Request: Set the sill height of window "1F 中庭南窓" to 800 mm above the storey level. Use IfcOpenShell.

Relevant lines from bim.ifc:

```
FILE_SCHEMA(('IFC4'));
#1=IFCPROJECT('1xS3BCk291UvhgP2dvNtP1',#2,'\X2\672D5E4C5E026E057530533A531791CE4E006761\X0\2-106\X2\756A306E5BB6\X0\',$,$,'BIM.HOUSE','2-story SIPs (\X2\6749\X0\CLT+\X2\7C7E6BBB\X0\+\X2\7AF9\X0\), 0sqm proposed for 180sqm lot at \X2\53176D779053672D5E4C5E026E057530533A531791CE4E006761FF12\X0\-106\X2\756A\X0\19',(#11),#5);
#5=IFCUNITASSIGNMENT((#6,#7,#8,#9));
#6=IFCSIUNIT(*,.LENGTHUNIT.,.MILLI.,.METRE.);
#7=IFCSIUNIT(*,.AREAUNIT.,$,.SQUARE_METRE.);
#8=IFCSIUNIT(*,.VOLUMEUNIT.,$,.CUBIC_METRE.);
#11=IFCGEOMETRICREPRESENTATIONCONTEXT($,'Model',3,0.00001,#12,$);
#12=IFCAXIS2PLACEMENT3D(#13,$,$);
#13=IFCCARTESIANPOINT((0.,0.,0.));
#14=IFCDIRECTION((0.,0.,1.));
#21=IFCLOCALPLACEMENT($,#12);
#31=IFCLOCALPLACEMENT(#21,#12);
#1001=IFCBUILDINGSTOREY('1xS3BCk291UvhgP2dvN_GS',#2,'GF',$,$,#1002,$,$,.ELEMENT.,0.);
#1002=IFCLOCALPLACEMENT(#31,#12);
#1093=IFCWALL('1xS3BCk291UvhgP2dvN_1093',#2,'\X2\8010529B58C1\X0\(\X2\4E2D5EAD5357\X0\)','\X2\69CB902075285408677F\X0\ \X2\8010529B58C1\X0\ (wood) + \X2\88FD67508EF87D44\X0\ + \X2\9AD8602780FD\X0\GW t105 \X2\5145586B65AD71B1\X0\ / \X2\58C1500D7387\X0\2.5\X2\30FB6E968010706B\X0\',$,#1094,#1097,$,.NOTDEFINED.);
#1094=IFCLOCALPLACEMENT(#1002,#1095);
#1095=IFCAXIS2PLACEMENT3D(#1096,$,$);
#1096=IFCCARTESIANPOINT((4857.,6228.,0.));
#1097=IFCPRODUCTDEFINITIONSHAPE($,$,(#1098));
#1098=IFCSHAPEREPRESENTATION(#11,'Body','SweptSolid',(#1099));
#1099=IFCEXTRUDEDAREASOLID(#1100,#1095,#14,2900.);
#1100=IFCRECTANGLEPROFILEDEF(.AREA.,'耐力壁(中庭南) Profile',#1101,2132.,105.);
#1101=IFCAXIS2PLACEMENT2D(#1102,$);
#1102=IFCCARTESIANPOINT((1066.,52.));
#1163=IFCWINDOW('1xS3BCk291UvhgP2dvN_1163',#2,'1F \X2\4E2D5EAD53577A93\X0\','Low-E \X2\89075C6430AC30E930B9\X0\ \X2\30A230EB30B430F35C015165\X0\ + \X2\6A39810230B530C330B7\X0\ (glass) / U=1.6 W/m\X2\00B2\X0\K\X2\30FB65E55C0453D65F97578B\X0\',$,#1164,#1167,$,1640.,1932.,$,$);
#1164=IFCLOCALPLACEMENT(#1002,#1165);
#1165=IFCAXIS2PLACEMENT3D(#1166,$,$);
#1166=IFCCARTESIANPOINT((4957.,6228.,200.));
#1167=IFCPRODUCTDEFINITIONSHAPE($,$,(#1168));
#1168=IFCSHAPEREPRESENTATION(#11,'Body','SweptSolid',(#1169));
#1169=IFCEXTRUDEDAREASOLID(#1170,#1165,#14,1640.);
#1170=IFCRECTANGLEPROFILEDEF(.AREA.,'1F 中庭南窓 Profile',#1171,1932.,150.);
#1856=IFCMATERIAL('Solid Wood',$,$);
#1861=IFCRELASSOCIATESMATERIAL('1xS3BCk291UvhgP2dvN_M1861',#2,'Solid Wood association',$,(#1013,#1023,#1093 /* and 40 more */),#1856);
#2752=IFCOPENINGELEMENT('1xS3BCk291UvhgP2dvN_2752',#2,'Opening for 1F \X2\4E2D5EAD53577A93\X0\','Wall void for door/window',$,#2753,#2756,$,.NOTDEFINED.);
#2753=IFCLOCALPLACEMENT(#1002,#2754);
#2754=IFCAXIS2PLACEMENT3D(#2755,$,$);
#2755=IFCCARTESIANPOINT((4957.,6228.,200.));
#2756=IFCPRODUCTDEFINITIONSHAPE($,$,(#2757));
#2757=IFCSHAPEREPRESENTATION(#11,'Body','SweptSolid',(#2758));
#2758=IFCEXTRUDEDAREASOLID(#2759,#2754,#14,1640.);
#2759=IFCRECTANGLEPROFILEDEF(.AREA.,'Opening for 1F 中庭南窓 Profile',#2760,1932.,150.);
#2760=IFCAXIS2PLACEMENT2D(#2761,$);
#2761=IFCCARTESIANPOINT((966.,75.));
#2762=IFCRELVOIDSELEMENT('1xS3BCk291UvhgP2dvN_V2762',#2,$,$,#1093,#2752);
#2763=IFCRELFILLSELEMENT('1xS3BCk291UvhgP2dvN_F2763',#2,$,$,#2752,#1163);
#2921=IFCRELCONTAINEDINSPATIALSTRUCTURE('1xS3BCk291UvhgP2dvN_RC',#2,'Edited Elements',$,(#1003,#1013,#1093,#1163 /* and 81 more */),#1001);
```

```python
import numpy as np
import ifcopenshell
import ifcopenshell.api.geometry
import ifcopenshell.geom
import ifcopenshell.util.element
import ifcopenshell.util.placement
import ifcopenshell.util.shape
import ifcopenshell.util.unit

model = ifcopenshell.open("bim.ifc")
unit_scale = ifcopenshell.util.unit.calculate_unit_scale(model)

window = model.by_guid("1xS3BCk291UvhgP2dvN_1163")
opening = window.FillsVoids[0].RelatingOpeningElement
storey = ifcopenshell.util.element.get_container(window, ifc_class="IfcBuildingStorey")
level = ifcopenshell.util.placement.get_local_placement(storey.ObjectPlacement)[2, 3]

# The opening's origin need not be at the sill, so measure its lowest point.
shape = ifcopenshell.geom.create_shape(ifcopenshell.geom.settings(), opening)
bottom = ifcopenshell.util.shape.get_shape_bottom_elevation(shape, shape.geometry) / unit_scale
dz = level + 0.8 / unit_scale - bottom

shift = np.array([0.0, 0.0, dz])
# The window is not placed relative to its opening, so move both.
for product in (opening, window):
    matrix = ifcopenshell.util.placement.get_local_placement(product.ObjectPlacement)
    matrix[:3, 3] += shift
    ifcopenshell.api.geometry.edit_object_placement(model, product=product, matrix=matrix, is_si=False)

print(f"moved by {dz * unit_scale:+.3f} m")

model.write("bim_rev.ifc")
```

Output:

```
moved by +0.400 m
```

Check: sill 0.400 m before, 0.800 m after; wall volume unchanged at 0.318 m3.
